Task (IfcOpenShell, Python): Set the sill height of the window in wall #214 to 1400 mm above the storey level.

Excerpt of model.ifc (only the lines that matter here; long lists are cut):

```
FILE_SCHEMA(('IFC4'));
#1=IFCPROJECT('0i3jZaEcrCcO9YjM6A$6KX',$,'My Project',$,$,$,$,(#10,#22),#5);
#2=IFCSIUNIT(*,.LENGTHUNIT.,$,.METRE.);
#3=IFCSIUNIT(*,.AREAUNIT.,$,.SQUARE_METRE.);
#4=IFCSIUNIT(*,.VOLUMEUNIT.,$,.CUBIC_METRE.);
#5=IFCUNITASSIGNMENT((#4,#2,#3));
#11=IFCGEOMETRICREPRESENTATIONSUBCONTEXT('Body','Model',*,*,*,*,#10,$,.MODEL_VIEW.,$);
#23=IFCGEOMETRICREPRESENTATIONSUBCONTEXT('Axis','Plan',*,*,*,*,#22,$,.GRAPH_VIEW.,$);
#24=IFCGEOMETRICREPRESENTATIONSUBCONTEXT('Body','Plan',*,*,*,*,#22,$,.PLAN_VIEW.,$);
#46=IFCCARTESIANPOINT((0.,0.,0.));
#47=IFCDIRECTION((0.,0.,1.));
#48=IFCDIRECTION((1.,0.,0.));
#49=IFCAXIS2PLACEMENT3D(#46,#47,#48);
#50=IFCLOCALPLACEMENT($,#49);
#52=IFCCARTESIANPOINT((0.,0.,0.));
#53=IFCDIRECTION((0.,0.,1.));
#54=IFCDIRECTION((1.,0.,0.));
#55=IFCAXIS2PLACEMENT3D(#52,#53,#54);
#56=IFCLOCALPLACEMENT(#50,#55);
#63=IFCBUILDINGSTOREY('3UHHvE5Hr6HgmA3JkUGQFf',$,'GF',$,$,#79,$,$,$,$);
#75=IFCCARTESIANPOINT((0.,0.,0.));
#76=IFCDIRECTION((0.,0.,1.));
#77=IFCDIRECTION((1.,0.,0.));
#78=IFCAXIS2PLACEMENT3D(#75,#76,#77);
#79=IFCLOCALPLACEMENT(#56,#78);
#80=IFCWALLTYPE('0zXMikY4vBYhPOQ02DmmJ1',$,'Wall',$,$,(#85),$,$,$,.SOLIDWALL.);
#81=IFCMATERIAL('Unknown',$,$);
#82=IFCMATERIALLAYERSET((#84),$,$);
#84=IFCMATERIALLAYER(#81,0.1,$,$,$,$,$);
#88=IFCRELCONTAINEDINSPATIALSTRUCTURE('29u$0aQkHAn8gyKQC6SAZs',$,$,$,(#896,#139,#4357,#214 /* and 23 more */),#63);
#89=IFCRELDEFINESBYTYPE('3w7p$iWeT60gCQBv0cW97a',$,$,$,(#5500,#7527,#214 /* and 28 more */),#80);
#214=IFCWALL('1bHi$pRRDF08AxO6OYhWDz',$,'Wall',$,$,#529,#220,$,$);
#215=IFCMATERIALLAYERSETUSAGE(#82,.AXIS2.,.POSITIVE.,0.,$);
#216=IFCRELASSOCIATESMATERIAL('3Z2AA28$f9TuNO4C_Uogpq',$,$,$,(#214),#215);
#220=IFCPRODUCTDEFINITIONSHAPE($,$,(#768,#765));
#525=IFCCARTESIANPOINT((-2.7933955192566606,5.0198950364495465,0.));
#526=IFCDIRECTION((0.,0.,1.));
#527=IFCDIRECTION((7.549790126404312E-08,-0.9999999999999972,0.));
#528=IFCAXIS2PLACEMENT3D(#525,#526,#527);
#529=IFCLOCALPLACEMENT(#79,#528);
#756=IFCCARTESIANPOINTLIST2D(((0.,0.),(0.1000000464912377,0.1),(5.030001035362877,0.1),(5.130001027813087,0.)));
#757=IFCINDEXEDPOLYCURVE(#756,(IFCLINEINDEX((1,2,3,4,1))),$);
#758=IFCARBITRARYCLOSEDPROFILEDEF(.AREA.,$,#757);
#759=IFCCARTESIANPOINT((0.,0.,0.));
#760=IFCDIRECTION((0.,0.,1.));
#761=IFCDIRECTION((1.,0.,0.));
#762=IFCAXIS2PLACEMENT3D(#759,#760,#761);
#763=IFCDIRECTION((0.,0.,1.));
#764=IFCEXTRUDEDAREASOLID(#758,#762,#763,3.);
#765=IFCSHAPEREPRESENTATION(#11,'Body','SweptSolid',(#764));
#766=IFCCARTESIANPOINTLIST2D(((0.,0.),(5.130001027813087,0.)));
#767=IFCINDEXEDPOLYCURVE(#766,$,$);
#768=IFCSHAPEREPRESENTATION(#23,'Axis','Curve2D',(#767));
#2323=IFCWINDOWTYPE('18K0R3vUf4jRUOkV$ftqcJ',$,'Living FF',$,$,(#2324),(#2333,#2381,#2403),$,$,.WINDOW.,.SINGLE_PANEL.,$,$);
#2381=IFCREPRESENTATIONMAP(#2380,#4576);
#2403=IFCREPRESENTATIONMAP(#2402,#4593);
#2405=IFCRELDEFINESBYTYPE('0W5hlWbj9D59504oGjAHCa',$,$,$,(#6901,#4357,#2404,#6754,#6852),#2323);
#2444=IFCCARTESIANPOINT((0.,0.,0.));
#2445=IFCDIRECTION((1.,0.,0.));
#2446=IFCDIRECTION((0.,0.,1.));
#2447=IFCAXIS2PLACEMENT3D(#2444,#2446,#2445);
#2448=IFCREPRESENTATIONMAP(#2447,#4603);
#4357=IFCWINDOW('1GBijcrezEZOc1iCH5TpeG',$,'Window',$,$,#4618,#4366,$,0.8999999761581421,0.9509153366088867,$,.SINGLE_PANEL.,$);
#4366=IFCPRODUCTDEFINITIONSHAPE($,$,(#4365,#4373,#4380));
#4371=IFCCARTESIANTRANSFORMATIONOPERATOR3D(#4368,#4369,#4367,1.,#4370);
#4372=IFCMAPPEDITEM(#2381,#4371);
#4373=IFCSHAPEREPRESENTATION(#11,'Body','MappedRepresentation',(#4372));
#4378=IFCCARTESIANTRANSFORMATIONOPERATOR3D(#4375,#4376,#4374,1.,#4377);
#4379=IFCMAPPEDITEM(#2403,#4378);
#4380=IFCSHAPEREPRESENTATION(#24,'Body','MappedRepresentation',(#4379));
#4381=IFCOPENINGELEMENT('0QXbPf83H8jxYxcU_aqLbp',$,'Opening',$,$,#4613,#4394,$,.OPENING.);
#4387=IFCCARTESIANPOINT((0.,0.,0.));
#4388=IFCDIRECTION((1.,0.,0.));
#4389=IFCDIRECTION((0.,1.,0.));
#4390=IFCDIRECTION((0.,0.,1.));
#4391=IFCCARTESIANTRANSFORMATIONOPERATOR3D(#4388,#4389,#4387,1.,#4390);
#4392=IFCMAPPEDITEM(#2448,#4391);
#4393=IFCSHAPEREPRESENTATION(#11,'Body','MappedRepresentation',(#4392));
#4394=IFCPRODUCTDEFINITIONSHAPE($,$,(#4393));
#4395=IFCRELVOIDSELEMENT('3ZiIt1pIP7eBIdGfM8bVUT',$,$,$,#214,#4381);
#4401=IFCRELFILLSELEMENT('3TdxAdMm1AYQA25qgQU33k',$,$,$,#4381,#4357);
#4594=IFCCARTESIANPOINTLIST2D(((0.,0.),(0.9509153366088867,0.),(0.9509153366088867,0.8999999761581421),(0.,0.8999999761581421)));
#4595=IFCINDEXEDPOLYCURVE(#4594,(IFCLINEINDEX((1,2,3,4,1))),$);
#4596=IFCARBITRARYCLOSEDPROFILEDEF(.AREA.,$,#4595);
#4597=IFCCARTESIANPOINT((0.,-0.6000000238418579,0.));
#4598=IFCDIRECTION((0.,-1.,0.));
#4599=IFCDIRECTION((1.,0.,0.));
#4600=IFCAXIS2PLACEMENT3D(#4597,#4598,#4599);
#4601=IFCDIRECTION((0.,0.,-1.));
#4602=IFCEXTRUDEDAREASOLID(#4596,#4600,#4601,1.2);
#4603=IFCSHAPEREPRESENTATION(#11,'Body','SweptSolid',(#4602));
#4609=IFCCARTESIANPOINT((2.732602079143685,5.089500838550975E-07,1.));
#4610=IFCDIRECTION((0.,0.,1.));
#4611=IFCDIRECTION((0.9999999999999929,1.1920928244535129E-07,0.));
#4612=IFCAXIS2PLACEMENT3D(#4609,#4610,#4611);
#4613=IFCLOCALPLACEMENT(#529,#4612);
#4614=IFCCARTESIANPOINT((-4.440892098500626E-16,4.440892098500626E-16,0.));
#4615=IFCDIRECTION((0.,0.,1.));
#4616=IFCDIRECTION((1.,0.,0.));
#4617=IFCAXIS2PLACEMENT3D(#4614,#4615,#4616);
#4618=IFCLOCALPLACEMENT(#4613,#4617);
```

```python
import numpy as np
import ifcopenshell
import ifcopenshell.api.geometry
import ifcopenshell.geom
import ifcopenshell.util.element
import ifcopenshell.util.placement
import ifcopenshell.util.shape
import ifcopenshell.util.unit

model = ifcopenshell.open("model.ifc")
unit_scale = ifcopenshell.util.unit.calculate_unit_scale(model)

window = model.by_guid("1GBijcrezEZOc1iCH5TpeG")
opening = window.FillsVoids[0].RelatingOpeningElement
storey = ifcopenshell.util.element.get_container(window, ifc_class="IfcBuildingStorey")
level = ifcopenshell.util.placement.get_local_placement(storey.ObjectPlacement)[2, 3]

# The opening's origin need not be at the sill, so measure its lowest point.
shape = ifcopenshell.geom.create_shape(ifcopenshell.geom.settings(), opening)
bottom = ifcopenshell.util.shape.get_shape_bottom_elevation(shape, shape.geometry) / unit_scale
dz = level + 1.4 / unit_scale - bottom

shift = np.array([0.0, 0.0, dz])
# The window is placed relative to its opening, so it follows when the opening moves.
matrix = ifcopenshell.util.placement.get_local_placement(opening.ObjectPlacement)
matrix[:3, 3] += shift
ifcopenshell.api.geometry.edit_object_placement(
    model, product=opening, matrix=matrix, is_si=False, should_transform_children=True
)

print(f"moved by {dz * unit_scale:+.3f} m")

model.write("model-out.ifc")
```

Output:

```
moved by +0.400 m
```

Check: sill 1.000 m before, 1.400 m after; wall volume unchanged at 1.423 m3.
